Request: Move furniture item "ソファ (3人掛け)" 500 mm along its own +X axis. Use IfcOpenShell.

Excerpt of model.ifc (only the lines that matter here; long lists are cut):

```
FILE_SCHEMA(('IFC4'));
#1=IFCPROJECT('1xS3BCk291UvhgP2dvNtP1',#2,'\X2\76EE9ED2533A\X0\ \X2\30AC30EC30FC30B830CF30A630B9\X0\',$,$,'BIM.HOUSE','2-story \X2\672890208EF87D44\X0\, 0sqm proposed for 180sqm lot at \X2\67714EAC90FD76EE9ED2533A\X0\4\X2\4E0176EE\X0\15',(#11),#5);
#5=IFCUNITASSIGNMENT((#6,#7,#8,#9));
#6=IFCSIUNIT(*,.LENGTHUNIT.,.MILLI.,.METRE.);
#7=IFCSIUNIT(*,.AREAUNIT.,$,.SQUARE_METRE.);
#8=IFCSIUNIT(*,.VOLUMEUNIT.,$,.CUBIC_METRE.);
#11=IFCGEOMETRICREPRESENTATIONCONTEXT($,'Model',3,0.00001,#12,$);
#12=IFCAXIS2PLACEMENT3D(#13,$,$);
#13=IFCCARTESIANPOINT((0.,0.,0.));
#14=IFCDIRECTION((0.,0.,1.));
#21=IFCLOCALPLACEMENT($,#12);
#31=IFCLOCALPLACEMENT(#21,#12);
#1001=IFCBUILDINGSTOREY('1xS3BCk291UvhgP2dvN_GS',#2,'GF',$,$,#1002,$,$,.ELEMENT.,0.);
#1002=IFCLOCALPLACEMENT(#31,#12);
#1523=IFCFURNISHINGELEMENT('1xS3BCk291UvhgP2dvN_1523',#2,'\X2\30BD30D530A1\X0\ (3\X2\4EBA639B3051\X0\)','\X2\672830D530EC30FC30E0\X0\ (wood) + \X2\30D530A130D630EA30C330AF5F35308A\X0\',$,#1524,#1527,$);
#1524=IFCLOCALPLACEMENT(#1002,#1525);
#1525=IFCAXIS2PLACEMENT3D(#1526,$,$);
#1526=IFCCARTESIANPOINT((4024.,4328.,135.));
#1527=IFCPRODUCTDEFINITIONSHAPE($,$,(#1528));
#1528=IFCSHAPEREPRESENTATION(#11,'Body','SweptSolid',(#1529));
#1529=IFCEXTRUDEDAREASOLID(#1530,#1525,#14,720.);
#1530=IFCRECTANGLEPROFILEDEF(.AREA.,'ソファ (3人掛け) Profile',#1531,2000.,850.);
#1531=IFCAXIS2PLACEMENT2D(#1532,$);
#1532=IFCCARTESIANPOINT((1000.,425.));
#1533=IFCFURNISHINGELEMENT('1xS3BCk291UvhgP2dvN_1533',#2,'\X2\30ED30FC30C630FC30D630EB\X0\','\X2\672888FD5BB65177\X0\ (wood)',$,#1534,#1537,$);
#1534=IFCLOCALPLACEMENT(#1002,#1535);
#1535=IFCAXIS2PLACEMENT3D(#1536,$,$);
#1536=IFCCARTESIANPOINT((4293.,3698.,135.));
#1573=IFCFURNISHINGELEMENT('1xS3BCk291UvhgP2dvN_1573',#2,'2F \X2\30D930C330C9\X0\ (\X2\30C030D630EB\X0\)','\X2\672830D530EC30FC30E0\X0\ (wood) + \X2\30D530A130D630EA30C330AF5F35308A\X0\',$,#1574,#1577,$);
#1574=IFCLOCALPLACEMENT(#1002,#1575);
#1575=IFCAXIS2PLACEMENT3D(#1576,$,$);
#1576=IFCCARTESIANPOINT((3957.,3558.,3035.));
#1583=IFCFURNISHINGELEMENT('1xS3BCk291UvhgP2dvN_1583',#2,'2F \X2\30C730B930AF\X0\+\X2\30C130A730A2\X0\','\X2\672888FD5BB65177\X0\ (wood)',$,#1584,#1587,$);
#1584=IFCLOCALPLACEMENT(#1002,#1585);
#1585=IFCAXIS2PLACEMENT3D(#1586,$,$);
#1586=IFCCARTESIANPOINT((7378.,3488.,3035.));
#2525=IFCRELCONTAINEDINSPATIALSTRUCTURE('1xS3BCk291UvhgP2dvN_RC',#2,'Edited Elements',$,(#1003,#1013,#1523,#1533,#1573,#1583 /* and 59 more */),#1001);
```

```python
import ifcopenshell
import ifcopenshell.api.geometry
import ifcopenshell.util.placement
import ifcopenshell.util.unit

model = ifcopenshell.open("model.ifc")
unit_scale = ifcopenshell.util.unit.calculate_unit_scale(model)

item = model.by_guid("1xS3BCk291UvhgP2dvN_1523")
matrix = ifcopenshell.util.placement.get_local_placement(item.ObjectPlacement)
matrix[:3, 3] += matrix[:3, 0] * 0.5 / unit_scale
ifcopenshell.api.geometry.edit_object_placement(model, product=item, matrix=matrix, is_si=False)

print(ifcopenshell.util.placement.get_local_placement(item.ObjectPlacement).round(3) + 0.0)

model.write("model_updated.ifc")
```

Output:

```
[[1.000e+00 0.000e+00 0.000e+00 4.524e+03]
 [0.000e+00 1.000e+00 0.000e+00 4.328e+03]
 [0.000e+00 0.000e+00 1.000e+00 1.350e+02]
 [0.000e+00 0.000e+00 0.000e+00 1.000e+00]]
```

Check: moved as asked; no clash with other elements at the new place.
